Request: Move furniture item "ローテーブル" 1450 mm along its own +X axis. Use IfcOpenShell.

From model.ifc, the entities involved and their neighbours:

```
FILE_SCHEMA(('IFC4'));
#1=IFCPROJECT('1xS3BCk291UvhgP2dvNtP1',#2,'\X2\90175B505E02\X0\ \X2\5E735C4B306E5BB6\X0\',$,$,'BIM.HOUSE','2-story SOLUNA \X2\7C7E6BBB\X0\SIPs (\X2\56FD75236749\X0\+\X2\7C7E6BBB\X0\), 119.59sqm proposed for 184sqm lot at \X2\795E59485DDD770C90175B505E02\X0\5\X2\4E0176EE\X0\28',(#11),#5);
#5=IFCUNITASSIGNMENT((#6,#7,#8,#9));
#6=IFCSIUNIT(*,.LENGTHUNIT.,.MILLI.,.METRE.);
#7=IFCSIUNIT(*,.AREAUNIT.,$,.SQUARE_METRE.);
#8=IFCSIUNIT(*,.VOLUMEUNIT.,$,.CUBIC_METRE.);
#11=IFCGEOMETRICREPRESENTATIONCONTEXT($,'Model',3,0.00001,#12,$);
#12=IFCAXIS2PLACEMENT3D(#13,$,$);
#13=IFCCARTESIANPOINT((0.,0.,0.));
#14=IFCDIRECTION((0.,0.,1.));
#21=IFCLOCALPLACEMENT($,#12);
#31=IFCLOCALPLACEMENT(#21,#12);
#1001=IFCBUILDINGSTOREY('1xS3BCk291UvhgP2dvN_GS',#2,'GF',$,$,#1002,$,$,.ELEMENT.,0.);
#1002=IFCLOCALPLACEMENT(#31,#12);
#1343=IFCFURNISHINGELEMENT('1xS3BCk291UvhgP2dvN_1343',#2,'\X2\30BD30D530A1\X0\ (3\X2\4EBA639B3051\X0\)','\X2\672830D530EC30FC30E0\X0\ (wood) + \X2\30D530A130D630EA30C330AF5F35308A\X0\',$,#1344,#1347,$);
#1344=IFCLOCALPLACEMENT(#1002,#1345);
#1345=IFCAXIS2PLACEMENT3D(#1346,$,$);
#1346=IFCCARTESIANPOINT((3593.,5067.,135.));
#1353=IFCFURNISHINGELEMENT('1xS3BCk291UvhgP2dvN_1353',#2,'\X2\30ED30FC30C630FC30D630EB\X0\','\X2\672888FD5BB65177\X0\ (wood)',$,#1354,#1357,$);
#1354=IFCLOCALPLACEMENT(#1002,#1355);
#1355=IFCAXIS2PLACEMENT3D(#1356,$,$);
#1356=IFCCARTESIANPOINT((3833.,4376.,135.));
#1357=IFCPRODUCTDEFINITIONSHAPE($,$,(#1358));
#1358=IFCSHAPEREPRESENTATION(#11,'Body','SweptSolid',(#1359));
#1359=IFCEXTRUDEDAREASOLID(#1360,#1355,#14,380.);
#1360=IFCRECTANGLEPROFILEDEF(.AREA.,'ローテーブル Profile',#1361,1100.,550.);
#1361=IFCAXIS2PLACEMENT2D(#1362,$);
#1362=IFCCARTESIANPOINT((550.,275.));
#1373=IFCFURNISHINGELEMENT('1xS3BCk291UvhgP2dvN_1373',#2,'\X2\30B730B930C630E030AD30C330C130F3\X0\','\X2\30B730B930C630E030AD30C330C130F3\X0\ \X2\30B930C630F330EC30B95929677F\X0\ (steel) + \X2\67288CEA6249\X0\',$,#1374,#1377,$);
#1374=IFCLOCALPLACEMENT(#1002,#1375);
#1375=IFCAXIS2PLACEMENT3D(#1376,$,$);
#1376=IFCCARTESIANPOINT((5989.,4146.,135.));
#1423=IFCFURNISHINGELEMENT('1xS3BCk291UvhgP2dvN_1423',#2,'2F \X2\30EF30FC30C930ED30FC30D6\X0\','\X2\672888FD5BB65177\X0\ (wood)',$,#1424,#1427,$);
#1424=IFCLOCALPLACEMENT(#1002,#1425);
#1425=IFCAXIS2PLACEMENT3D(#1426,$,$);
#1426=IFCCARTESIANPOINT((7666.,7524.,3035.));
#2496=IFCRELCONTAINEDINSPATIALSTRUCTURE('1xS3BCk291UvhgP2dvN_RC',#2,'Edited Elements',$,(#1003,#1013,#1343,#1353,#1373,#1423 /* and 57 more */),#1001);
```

```python
import ifcopenshell
import ifcopenshell.api.geometry
import ifcopenshell.util.placement
import ifcopenshell.util.unit

model = ifcopenshell.open("model.ifc")
unit_scale = ifcopenshell.util.unit.calculate_unit_scale(model)

item = model.by_guid("1xS3BCk291UvhgP2dvN_1353")
matrix = ifcopenshell.util.placement.get_local_placement(item.ObjectPlacement)
matrix[:3, 3] += matrix[:3, 0] * 1.45 / unit_scale
ifcopenshell.api.geometry.edit_object_placement(model, product=item, matrix=matrix, is_si=False)

print(ifcopenshell.util.placement.get_local_placement(item.ObjectPlacement).round(3) + 0.0)

model.write("model_rev.ifc")
```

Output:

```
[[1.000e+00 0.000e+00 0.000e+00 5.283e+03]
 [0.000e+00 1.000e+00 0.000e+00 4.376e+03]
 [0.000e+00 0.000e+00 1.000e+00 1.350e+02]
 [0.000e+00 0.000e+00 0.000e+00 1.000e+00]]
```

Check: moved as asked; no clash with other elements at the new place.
